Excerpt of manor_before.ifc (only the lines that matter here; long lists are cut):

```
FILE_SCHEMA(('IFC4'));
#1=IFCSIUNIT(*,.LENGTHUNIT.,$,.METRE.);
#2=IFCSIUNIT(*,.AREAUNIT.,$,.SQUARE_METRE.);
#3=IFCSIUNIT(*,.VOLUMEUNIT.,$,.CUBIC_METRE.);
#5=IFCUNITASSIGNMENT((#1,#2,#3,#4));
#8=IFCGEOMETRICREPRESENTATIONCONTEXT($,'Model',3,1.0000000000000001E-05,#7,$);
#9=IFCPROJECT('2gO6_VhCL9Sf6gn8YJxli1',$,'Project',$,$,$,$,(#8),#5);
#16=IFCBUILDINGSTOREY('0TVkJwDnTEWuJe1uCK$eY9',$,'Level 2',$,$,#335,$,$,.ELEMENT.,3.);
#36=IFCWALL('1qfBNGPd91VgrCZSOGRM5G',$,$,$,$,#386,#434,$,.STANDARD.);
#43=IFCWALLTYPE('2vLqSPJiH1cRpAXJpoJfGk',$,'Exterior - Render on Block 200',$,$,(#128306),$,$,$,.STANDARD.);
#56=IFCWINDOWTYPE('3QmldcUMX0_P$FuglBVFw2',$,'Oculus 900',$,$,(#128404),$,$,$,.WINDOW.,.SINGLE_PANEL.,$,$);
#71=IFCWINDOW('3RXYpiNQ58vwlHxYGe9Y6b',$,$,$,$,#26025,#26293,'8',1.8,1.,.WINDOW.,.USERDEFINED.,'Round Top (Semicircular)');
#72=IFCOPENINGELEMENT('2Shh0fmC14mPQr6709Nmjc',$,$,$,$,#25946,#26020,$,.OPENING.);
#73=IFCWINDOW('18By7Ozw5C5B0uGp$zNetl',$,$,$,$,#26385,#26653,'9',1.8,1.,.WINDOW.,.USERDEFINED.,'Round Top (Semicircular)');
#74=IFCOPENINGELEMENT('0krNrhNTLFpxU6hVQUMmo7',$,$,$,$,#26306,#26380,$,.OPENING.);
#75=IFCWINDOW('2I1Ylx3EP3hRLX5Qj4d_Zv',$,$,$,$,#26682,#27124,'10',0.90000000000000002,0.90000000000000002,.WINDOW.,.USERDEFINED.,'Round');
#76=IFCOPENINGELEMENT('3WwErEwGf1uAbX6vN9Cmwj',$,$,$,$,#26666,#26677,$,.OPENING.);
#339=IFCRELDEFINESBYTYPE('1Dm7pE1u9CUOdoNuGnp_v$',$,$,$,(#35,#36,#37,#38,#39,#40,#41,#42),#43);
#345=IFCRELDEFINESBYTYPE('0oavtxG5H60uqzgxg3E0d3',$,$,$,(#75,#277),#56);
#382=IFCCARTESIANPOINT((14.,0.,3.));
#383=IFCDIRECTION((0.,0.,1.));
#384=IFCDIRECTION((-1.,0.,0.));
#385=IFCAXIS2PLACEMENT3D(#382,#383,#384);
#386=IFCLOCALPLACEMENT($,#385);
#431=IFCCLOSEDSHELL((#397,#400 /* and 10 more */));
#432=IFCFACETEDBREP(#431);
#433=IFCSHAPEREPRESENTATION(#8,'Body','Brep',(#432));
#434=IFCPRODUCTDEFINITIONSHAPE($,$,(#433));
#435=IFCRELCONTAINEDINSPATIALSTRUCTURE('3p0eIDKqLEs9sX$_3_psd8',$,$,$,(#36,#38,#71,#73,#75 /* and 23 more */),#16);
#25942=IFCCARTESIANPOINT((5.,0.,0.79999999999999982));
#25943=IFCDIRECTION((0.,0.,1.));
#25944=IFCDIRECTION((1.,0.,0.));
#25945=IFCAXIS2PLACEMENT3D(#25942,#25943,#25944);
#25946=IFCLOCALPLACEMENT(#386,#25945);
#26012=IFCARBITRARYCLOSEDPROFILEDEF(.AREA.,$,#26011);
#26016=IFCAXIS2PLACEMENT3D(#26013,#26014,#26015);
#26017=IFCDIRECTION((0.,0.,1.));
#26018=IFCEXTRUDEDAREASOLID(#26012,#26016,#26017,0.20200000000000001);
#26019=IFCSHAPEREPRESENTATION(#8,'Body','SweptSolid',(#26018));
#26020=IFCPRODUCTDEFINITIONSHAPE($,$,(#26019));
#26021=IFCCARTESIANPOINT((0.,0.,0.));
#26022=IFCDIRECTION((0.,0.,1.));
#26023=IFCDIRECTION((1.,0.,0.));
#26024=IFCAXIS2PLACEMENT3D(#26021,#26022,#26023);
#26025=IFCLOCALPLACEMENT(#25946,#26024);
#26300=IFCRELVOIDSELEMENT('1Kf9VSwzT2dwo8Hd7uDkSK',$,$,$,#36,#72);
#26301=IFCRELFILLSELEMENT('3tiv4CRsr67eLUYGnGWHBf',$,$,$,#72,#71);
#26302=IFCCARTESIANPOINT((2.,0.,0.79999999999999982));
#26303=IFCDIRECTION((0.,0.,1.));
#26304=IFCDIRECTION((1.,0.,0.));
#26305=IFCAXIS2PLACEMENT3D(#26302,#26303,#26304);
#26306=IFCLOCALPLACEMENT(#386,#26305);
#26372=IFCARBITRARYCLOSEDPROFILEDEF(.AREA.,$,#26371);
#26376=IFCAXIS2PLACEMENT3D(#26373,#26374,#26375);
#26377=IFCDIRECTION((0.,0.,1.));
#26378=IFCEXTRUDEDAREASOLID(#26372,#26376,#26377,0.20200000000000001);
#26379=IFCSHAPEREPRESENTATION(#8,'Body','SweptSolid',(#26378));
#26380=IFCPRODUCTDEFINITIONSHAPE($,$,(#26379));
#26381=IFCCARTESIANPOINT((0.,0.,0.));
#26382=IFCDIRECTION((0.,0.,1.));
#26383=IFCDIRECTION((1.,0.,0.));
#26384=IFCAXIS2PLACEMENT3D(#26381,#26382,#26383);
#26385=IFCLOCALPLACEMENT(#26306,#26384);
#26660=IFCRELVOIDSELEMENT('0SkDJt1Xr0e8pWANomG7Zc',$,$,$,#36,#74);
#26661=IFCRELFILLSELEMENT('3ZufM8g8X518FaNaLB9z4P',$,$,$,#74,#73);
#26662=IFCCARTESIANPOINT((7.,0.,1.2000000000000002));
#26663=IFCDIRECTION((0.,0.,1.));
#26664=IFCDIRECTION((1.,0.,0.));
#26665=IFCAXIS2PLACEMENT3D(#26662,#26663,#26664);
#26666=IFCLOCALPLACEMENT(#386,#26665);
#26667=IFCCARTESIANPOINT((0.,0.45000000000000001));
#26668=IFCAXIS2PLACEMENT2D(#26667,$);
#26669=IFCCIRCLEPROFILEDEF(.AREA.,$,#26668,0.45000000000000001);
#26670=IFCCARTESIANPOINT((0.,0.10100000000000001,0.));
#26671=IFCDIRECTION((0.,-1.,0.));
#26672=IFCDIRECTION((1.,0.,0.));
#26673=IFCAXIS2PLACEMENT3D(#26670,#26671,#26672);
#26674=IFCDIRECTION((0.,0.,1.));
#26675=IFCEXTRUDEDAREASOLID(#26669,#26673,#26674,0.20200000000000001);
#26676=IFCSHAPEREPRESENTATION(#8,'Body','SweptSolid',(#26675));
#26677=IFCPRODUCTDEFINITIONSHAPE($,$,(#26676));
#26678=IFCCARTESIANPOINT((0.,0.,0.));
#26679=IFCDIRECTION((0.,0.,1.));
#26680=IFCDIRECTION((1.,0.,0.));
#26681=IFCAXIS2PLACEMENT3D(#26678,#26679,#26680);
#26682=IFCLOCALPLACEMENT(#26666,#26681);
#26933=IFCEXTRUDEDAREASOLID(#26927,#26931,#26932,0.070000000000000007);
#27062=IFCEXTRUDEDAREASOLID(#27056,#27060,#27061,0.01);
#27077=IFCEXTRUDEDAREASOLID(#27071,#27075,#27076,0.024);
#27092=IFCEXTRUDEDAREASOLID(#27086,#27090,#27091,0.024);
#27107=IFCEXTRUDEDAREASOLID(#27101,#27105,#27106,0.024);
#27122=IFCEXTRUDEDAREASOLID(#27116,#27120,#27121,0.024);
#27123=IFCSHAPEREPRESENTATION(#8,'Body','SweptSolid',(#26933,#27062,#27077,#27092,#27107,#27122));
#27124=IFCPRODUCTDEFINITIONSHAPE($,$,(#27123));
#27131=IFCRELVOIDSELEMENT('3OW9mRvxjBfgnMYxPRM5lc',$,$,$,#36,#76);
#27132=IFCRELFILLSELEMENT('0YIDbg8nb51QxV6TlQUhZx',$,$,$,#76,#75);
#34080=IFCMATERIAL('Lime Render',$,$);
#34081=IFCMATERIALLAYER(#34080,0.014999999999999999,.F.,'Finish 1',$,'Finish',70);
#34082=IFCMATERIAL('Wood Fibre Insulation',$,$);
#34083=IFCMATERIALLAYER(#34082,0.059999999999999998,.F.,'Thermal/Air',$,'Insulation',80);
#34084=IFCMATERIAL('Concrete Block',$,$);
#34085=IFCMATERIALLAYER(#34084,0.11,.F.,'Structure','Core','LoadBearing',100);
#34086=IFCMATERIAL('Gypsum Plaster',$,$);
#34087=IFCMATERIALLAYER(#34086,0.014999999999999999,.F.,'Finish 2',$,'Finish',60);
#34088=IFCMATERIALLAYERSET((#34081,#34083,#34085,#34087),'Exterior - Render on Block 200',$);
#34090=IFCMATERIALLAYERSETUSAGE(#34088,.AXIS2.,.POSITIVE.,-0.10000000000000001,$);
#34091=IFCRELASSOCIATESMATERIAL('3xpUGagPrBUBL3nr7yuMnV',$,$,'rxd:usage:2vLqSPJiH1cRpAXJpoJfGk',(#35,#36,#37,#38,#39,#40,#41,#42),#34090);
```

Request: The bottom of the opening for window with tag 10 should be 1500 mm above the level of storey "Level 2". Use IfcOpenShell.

```python
import numpy as np
import ifcopenshell
import ifcopenshell.api.geometry
import ifcopenshell.geom
import ifcopenshell.util.element
import ifcopenshell.util.placement
import ifcopenshell.util.shape
import ifcopenshell.util.unit

model = ifcopenshell.open("manor_before.ifc")
unit_scale = ifcopenshell.util.unit.calculate_unit_scale(model)

window = model.by_guid("2I1Ylx3EP3hRLX5Qj4d_Zv")
opening = window.FillsVoids[0].RelatingOpeningElement
storey = ifcopenshell.util.element.get_container(window, ifc_class="IfcBuildingStorey")
level = ifcopenshell.util.placement.get_local_placement(storey.ObjectPlacement)[2, 3]

# The opening's origin need not be at the sill, so measure its lowest point.
shape = ifcopenshell.geom.create_shape(ifcopenshell.geom.settings(), opening)
bottom = ifcopenshell.util.shape.get_shape_bottom_elevation(shape, shape.geometry) / unit_scale
dz = level + 1.5 / unit_scale - bottom

shift = np.array([0.0, 0.0, dz])
# The window is placed relative to its opening, so it follows when the opening moves.
matrix = ifcopenshell.util.placement.get_local_placement(opening.ObjectPlacement)
matrix[:3, 3] += shift
ifcopenshell.api.geometry.edit_object_placement(
    model, product=opening, matrix=matrix, is_si=False, should_transform_children=True
)

print(f"moved by {dz * unit_scale:+.3f} m")

model.write("manor_before_updated.ifc")
```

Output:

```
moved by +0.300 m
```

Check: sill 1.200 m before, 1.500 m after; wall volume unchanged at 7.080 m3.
